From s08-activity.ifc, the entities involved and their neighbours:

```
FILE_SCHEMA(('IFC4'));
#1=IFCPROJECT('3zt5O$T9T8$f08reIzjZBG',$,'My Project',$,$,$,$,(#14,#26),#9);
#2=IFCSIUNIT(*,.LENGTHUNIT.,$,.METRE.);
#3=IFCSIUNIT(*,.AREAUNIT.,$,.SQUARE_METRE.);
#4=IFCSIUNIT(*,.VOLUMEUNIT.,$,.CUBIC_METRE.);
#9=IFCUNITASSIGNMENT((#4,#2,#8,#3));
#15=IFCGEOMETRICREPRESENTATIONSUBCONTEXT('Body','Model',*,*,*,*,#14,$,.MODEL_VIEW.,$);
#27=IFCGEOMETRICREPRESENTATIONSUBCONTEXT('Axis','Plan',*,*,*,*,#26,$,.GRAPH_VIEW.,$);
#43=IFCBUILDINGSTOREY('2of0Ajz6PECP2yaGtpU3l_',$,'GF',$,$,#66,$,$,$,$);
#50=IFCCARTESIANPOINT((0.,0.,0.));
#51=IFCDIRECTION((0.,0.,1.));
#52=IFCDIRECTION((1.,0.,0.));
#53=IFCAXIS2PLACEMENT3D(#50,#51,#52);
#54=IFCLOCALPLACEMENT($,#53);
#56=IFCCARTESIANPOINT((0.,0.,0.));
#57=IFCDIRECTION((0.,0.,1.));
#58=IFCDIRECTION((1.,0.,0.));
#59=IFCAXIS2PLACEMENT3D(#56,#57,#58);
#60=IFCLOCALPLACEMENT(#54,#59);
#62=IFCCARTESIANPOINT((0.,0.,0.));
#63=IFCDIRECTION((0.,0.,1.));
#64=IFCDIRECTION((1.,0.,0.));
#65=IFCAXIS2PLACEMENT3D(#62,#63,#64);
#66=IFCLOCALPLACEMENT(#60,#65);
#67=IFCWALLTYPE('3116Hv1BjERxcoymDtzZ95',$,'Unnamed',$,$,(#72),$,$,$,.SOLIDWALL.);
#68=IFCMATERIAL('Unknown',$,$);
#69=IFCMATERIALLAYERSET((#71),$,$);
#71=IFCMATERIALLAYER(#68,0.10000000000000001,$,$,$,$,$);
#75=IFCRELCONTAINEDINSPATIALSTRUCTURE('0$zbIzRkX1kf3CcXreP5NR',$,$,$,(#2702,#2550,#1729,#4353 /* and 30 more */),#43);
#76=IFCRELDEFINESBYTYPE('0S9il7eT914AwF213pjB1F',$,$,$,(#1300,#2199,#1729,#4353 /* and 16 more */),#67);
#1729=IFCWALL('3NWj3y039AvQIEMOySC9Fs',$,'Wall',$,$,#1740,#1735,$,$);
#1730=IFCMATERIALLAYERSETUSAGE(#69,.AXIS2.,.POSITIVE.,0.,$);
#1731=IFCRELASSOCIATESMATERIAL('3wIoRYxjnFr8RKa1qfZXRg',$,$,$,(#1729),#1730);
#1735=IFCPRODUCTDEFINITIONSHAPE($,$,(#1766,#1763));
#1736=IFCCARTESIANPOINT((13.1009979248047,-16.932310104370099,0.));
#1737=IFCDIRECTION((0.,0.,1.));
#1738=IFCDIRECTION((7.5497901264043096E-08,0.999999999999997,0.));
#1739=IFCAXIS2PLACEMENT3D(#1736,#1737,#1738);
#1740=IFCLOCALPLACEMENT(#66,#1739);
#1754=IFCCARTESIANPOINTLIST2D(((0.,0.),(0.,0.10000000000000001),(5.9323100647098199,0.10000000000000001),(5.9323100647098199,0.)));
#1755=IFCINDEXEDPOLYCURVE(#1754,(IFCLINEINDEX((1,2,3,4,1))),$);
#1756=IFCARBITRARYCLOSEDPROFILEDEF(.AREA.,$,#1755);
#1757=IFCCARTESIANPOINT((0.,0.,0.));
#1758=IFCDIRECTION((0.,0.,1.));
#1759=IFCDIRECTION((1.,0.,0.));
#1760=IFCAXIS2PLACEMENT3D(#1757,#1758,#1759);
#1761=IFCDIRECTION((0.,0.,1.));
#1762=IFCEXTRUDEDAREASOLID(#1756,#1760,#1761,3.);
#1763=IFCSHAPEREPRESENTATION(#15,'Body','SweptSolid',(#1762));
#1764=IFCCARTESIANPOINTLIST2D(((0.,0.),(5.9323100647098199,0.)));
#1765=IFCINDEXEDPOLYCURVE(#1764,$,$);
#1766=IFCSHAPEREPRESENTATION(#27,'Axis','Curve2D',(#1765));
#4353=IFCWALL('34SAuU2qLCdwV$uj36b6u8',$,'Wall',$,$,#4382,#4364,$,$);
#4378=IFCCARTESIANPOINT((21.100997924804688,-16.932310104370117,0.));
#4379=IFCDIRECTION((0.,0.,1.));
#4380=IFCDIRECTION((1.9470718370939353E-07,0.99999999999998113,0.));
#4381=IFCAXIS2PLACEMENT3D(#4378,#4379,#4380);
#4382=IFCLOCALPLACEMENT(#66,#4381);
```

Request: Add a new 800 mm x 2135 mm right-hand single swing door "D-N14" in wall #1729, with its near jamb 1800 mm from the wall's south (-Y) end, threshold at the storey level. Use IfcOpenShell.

```python
import numpy as np
import ifcopenshell
import ifcopenshell.api.feature
import ifcopenshell.api.geometry
import ifcopenshell.api.root
import ifcopenshell.api.spatial
import ifcopenshell.geom
import ifcopenshell.util.element
import ifcopenshell.util.placement
import ifcopenshell.util.representation
import ifcopenshell.util.shape
import ifcopenshell.util.unit

model = ifcopenshell.open("s08-activity.ifc")
unit_scale = ifcopenshell.util.unit.calculate_unit_scale(model)
settings = ifcopenshell.geom.settings()


def volume(element):
    """Net volume in cubic metres, openings subtracted."""
    shape = ifcopenshell.geom.create_shape(settings, element)
    return ifcopenshell.util.shape.get_volume(shape.geometry)


wall = model.by_guid("3NWj3y039AvQIEMOySC9Fs")
storey = ifcopenshell.util.element.get_container(wall, ifc_class="IfcBuildingStorey")
context = ifcopenshell.util.representation.get_context(model, "Model", "Body", "MODEL_VIEW")
before = volume(wall)

width, height, from_end, sill = 0.8, 2.135, 1.8, 0.0  # metres

# The wall runs along its own X axis, and the end named is its -X end.
wall_shape = ifcopenshell.geom.create_shape(settings, wall)
x, y, z = ifcopenshell.util.shape.get_vertices(wall_shape.geometry).T
start = x.min() + from_end
face, thickness = float(y.min()), float(y.max() - y.min())
wall_matrix = ifcopenshell.util.placement.get_local_placement(wall.ObjectPlacement)
level = ifcopenshell.util.placement.get_local_placement(storey.ObjectPlacement)[2, 3]


def in_wall(x, y):
    """Placement at x, y metres in the wall's axes, at sill height."""
    matrix = wall_matrix.copy()
    matrix[:, 3] = wall_matrix @ np.array([x / unit_scale, y / unit_scale, 0.0, 1.0])
    matrix[2, 3] = level + sill / unit_scale
    return matrix


# Opening: a box that overshoots both wall faces by 50 mm.
opening = ifcopenshell.api.root.create_entity(model, ifc_class="IfcOpeningElement", predefined_type="OPENING")
box = ifcopenshell.api.geometry.add_wall_representation(
    model, context=context, length=width, height=height, thickness=thickness + 0.1
)
ifcopenshell.api.geometry.assign_representation(model, product=opening, representation=box)
ifcopenshell.api.geometry.edit_object_placement(model, product=opening, matrix=in_wall(start, face - 0.05), is_si=False)
ifcopenshell.api.feature.add_feature(model, feature=opening, element=wall)

door = ifcopenshell.api.root.create_entity(model, ifc_class="IfcDoor", name="D-N14", predefined_type="DOOR")
door.OverallWidth, door.OverallHeight = width / unit_scale, height / unit_scale
door.OperationType = "SINGLE_SWING_RIGHT"
body = ifcopenshell.api.geometry.add_door_representation(
    model,
    context=context,
    overall_width=door.OverallWidth,
    overall_height=door.OverallHeight,
    operation_type="SINGLE_SWING_RIGHT",
    lining_properties={"LiningDepth": thickness / unit_scale, "ThresholdDepth": thickness / unit_scale},
)
ifcopenshell.api.geometry.assign_representation(model, product=door, representation=body)
ifcopenshell.api.spatial.assign_container(model, products=[door], relating_structure=storey)
ifcopenshell.api.feature.add_filling(model, opening=opening, element=door)

# The lining spans the wall, so the door starts at the wall face.
ifcopenshell.api.geometry.edit_object_placement(model, product=door, matrix=in_wall(start, face), is_si=False)

after = volume(wall)

print(f"wall volume {before:.3f} -> {after:.3f} m3")

model.write("s08-activity_v2.ifc")
```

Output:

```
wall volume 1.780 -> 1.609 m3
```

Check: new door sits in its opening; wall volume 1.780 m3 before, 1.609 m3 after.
